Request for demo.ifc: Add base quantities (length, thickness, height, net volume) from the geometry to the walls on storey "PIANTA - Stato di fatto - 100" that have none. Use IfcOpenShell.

First a look at what the model holds.

```python
import ifcopenshell
import ifcopenshell.util.element
import ifcopenshell.util.unit

model = ifcopenshell.open("demo.ifc")
print(model.schema)
for unit_type in ("LENGTHUNIT", "AREAUNIT", "VOLUMEUNIT"):
    print(unit_type, ifcopenshell.util.unit.calculate_unit_scale(model, unit_type))
storey = next(s for s in model.by_type("IfcBuildingStorey") if s.Name == "PIANTA - Stato di fatto - 100")
walls = [e for e in ifcopenshell.util.element.get_decomposition(storey) if e.is_a("IfcWall")]
for e in sorted(walls, key=lambda e: e.id()):
    print(e.id(), e.is_a(), e.Name, list(ifcopenshell.util.element.get_psets(e, qtos_only=True)), sep=" | ")
```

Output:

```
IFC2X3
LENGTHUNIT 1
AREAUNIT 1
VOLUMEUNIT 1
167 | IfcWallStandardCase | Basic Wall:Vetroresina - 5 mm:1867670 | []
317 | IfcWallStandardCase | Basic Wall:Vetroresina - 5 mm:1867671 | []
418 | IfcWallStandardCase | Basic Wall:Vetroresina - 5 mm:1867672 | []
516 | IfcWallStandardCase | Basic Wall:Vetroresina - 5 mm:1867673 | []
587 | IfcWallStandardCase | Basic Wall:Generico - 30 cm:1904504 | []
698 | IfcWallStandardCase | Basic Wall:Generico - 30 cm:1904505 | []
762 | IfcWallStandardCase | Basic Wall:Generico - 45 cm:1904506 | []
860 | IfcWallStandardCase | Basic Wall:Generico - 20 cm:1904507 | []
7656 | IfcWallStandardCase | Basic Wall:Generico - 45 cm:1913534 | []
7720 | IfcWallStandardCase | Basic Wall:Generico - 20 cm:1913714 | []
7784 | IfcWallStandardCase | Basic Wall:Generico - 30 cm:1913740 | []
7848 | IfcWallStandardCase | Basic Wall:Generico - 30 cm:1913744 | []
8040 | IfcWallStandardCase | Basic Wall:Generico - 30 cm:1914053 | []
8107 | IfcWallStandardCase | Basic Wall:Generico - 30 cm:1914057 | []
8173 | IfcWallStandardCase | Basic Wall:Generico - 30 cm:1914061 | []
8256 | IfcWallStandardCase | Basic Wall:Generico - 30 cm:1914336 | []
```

```python
import ifcopenshell
import ifcopenshell.api.pset
import ifcopenshell.geom
import ifcopenshell.util.element
import ifcopenshell.util.shape
import ifcopenshell.util.unit

model = ifcopenshell.open("demo.ifc")
unit_scale = ifcopenshell.util.unit.calculate_unit_scale(model)
volume_scale = ifcopenshell.util.unit.calculate_unit_scale(model, "VOLUMEUNIT")
settings = ifcopenshell.geom.settings()

storey = next(s for s in model.by_type("IfcBuildingStorey") if s.Name == "PIANTA - Stato di fatto - 100")
walls = [e for e in ifcopenshell.util.element.get_decomposition(storey) if e.is_a("IfcWall")]

for e in sorted(walls, key=lambda e: e.id()):
    if ifcopenshell.util.element.get_psets(e, qtos_only=True, should_inherit=False):
        continue
    # Geometry comes back in metres, in the element's own axes.
    shape = ifcopenshell.geom.create_shape(settings, e)
    values = {
        "Length": ifcopenshell.util.shape.get_x(shape.geometry) / unit_scale,
        "Width": ifcopenshell.util.shape.get_y(shape.geometry) / unit_scale,
        "Height": ifcopenshell.util.shape.get_z(shape.geometry) / unit_scale,
        "NetVolume": ifcopenshell.util.shape.get_volume(shape.geometry) / volume_scale,
    }
    qto = ifcopenshell.api.pset.add_qto(model, product=e, name="BaseQuantities")
    ifcopenshell.api.pset.edit_qto(model, qto=qto, properties=values)
    print(e.id(), {k: round(v, 3) for k, v in values.items()})

model.write("demo-out.ifc")
```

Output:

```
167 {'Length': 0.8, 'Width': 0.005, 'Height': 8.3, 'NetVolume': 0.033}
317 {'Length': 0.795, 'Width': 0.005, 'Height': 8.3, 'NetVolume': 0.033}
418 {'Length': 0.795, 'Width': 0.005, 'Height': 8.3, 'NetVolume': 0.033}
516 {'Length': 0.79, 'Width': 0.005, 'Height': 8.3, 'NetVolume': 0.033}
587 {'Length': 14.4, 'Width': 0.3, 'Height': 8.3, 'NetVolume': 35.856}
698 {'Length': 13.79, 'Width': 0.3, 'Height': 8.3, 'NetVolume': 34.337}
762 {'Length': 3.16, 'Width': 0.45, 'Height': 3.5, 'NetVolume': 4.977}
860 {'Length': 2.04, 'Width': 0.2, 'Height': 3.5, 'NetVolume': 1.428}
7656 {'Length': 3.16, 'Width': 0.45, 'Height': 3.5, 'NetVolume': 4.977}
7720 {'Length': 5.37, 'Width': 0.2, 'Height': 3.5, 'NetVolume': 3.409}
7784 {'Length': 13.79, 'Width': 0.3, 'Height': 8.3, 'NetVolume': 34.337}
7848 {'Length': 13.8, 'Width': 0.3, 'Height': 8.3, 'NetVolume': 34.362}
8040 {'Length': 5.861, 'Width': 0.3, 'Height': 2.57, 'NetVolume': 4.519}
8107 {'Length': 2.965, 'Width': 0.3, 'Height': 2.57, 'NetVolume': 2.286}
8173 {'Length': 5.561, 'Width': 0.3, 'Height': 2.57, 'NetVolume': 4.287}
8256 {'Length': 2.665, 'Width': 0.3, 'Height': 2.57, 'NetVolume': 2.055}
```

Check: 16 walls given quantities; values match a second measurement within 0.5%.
